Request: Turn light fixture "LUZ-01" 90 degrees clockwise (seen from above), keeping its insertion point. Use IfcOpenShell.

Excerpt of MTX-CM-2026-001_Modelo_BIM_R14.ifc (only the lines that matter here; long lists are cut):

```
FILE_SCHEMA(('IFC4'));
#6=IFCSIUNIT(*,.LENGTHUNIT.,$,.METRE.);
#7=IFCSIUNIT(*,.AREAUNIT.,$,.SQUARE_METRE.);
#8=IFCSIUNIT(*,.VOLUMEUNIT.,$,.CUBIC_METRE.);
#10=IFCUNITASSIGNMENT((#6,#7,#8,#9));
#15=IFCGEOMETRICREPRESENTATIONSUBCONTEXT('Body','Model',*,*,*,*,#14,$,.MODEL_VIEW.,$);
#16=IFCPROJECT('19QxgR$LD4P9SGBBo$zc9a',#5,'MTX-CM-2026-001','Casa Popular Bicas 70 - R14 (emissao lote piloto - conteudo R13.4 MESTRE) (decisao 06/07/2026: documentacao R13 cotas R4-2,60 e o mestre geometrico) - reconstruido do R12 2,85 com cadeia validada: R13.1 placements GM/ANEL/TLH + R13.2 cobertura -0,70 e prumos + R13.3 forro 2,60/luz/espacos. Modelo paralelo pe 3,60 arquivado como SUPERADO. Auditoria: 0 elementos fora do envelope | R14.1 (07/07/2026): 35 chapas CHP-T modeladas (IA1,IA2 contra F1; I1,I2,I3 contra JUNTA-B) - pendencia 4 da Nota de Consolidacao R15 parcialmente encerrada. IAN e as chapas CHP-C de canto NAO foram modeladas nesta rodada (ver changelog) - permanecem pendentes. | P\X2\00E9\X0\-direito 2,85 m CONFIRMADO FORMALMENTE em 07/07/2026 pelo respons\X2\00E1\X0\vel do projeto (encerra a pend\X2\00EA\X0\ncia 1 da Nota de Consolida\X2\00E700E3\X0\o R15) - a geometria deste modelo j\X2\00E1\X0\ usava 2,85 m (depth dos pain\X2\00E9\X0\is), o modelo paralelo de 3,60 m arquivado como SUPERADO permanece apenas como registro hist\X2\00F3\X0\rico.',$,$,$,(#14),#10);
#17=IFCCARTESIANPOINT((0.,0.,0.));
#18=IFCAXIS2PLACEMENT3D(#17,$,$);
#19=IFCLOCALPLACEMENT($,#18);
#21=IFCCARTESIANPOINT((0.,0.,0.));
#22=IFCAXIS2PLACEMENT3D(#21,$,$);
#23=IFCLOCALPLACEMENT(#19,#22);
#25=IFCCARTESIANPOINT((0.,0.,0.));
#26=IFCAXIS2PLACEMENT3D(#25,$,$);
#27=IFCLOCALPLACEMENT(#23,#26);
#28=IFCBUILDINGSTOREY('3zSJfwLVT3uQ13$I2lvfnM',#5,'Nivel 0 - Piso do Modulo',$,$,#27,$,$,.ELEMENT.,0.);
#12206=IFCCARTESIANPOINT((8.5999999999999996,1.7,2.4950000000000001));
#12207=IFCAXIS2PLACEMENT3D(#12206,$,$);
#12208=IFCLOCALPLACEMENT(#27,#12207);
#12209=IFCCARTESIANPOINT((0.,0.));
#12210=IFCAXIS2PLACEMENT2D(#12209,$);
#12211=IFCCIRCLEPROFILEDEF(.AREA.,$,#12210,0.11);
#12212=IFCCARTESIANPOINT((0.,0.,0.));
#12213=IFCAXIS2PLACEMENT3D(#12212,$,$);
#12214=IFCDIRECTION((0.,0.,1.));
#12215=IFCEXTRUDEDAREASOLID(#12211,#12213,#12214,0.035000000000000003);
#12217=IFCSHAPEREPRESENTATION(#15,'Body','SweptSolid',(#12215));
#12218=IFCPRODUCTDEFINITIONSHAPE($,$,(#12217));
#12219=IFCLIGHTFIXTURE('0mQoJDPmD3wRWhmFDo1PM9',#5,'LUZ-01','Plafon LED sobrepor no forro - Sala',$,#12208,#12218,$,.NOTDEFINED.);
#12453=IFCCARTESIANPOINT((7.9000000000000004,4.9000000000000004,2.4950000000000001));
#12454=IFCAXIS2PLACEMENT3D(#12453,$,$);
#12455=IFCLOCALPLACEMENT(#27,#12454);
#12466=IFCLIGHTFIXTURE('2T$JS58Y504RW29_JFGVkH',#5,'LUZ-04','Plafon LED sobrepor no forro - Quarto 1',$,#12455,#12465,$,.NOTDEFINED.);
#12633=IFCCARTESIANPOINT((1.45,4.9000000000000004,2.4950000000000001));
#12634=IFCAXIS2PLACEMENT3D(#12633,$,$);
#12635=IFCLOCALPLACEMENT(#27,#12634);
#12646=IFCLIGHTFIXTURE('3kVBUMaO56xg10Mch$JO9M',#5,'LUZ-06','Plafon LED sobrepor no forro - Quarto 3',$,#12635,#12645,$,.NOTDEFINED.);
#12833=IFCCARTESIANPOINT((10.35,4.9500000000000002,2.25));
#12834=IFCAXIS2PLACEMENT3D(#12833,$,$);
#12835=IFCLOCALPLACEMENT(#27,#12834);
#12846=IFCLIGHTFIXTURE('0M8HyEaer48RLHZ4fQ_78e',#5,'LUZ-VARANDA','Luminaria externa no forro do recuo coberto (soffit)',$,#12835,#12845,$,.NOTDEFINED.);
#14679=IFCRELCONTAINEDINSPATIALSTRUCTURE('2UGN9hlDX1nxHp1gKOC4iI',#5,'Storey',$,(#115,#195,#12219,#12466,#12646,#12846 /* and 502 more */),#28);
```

```python
import ifcopenshell
import ifcopenshell.api.geometry
import ifcopenshell.util.placement

model = ifcopenshell.open("MTX-CM-2026-001_Modelo_BIM_R14.ifc")

item = model.by_guid("0mQoJDPmD3wRWhmFDo1PM9")
matrix = ifcopenshell.util.placement.get_local_placement(item.ObjectPlacement)
matrix = matrix @ ifcopenshell.util.placement.rotation(-90, "Z")
ifcopenshell.api.geometry.edit_object_placement(model, product=item, matrix=matrix, is_si=False)

print(ifcopenshell.util.placement.get_local_placement(item.ObjectPlacement).round(3) + 0.0)

model.write("MTX-CM-2026-001_Modelo_BIM_R14_updated.ifc")
```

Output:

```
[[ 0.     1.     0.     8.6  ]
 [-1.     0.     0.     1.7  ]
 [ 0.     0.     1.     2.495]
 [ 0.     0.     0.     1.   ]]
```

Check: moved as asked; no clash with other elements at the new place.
